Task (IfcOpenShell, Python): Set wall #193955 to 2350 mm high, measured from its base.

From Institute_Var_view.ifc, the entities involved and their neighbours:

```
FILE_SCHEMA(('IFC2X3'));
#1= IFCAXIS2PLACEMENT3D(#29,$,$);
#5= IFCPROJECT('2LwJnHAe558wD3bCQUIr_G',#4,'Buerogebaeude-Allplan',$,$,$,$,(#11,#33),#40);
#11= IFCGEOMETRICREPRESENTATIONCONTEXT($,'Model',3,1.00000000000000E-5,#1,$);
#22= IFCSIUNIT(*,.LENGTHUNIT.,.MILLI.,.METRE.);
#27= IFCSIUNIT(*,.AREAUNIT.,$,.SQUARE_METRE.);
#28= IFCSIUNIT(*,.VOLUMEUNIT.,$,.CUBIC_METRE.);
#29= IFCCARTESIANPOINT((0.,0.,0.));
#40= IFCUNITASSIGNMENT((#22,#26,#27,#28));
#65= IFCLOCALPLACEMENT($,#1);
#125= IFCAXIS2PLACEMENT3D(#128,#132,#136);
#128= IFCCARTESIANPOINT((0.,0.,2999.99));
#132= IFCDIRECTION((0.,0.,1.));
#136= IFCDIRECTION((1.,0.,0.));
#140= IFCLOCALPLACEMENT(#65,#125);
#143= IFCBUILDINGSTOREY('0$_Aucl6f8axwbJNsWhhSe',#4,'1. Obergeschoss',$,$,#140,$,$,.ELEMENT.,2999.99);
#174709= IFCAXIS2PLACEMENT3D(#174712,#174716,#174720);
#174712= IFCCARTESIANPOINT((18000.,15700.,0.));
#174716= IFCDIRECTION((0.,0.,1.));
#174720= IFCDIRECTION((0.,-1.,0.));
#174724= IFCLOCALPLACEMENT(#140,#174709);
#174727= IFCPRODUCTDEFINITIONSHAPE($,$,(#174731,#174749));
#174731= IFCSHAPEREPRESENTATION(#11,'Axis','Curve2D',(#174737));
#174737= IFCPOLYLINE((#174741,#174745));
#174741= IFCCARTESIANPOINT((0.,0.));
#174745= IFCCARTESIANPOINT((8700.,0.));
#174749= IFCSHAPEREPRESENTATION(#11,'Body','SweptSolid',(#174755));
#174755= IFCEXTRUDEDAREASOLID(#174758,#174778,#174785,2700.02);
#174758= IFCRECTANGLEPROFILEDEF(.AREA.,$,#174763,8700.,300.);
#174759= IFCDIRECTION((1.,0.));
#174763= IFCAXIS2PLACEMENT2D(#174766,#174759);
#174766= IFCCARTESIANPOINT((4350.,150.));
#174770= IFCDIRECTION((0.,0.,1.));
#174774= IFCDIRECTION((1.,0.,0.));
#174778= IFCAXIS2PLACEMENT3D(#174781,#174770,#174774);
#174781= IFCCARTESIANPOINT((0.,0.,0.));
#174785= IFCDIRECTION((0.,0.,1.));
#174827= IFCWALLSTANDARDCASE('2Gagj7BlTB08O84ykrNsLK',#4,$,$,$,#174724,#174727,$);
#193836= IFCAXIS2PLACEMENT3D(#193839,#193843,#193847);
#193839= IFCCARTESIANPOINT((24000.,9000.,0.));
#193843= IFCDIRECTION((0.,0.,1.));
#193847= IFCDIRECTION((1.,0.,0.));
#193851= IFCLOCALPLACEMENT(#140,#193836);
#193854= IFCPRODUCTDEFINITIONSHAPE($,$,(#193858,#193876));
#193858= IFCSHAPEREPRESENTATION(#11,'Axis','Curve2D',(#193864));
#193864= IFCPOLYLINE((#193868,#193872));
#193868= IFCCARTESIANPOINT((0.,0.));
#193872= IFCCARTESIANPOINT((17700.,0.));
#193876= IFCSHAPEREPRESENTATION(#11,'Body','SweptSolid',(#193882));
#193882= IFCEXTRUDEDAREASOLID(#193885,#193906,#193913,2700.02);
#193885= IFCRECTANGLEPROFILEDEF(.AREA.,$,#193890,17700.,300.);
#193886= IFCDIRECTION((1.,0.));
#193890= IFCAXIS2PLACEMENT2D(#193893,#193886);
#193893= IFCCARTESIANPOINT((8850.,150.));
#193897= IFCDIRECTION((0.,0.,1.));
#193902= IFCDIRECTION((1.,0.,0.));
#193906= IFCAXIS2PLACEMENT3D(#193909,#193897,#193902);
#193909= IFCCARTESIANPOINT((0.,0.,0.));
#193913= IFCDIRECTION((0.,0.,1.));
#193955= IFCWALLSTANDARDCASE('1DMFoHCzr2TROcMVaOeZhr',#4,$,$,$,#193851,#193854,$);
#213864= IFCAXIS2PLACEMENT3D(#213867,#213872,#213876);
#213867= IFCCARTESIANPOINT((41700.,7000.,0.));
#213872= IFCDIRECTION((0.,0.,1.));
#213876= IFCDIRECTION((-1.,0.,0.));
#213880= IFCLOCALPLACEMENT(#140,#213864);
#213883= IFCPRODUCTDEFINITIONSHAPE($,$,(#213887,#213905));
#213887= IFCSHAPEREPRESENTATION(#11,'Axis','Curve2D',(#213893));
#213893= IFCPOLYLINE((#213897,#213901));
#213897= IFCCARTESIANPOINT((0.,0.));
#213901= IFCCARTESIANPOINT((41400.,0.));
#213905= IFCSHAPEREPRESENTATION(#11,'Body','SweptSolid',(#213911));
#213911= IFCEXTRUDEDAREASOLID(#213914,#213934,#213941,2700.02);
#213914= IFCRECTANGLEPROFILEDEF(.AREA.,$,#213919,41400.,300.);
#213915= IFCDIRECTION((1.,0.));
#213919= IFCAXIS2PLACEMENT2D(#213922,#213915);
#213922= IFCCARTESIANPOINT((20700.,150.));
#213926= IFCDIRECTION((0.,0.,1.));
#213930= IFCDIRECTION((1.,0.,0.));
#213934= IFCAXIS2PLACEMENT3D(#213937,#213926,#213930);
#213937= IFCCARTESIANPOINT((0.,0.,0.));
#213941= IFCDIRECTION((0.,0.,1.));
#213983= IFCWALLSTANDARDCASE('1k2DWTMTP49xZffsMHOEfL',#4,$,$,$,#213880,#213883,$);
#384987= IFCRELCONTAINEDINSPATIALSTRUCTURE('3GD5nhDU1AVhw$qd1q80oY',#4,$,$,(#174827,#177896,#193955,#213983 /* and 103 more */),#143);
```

```python
import ifcopenshell
import ifcopenshell.geom
import ifcopenshell.util.shape
import ifcopenshell.util.unit

model = ifcopenshell.open("Institute_Var_view.ifc")
unit_scale = ifcopenshell.util.unit.calculate_unit_scale(model)
settings = ifcopenshell.geom.settings()


def volume(element):
    """Net volume in cubic metres, openings subtracted."""
    shape = ifcopenshell.geom.create_shape(settings, element)
    return ifcopenshell.util.shape.get_volume(shape.geometry)


wall = model.by_guid("1DMFoHCzr2TROcMVaOeZhr")
before = volume(wall)

body = next(r for r in wall.Representation.Representations if r.RepresentationIdentifier == "Body")
solid = body.Items[0]
old_height = solid.Depth
solid.Depth = 2.35 / unit_scale
after = volume(wall)

print(f"height {old_height:g} -> {solid.Depth:g}, volume {before:.3f} -> {after:.3f} m3")

model.write("Institute_Var_view_edited.ifc")
```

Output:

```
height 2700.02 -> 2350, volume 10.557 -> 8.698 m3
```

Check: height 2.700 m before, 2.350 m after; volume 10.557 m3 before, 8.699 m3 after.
